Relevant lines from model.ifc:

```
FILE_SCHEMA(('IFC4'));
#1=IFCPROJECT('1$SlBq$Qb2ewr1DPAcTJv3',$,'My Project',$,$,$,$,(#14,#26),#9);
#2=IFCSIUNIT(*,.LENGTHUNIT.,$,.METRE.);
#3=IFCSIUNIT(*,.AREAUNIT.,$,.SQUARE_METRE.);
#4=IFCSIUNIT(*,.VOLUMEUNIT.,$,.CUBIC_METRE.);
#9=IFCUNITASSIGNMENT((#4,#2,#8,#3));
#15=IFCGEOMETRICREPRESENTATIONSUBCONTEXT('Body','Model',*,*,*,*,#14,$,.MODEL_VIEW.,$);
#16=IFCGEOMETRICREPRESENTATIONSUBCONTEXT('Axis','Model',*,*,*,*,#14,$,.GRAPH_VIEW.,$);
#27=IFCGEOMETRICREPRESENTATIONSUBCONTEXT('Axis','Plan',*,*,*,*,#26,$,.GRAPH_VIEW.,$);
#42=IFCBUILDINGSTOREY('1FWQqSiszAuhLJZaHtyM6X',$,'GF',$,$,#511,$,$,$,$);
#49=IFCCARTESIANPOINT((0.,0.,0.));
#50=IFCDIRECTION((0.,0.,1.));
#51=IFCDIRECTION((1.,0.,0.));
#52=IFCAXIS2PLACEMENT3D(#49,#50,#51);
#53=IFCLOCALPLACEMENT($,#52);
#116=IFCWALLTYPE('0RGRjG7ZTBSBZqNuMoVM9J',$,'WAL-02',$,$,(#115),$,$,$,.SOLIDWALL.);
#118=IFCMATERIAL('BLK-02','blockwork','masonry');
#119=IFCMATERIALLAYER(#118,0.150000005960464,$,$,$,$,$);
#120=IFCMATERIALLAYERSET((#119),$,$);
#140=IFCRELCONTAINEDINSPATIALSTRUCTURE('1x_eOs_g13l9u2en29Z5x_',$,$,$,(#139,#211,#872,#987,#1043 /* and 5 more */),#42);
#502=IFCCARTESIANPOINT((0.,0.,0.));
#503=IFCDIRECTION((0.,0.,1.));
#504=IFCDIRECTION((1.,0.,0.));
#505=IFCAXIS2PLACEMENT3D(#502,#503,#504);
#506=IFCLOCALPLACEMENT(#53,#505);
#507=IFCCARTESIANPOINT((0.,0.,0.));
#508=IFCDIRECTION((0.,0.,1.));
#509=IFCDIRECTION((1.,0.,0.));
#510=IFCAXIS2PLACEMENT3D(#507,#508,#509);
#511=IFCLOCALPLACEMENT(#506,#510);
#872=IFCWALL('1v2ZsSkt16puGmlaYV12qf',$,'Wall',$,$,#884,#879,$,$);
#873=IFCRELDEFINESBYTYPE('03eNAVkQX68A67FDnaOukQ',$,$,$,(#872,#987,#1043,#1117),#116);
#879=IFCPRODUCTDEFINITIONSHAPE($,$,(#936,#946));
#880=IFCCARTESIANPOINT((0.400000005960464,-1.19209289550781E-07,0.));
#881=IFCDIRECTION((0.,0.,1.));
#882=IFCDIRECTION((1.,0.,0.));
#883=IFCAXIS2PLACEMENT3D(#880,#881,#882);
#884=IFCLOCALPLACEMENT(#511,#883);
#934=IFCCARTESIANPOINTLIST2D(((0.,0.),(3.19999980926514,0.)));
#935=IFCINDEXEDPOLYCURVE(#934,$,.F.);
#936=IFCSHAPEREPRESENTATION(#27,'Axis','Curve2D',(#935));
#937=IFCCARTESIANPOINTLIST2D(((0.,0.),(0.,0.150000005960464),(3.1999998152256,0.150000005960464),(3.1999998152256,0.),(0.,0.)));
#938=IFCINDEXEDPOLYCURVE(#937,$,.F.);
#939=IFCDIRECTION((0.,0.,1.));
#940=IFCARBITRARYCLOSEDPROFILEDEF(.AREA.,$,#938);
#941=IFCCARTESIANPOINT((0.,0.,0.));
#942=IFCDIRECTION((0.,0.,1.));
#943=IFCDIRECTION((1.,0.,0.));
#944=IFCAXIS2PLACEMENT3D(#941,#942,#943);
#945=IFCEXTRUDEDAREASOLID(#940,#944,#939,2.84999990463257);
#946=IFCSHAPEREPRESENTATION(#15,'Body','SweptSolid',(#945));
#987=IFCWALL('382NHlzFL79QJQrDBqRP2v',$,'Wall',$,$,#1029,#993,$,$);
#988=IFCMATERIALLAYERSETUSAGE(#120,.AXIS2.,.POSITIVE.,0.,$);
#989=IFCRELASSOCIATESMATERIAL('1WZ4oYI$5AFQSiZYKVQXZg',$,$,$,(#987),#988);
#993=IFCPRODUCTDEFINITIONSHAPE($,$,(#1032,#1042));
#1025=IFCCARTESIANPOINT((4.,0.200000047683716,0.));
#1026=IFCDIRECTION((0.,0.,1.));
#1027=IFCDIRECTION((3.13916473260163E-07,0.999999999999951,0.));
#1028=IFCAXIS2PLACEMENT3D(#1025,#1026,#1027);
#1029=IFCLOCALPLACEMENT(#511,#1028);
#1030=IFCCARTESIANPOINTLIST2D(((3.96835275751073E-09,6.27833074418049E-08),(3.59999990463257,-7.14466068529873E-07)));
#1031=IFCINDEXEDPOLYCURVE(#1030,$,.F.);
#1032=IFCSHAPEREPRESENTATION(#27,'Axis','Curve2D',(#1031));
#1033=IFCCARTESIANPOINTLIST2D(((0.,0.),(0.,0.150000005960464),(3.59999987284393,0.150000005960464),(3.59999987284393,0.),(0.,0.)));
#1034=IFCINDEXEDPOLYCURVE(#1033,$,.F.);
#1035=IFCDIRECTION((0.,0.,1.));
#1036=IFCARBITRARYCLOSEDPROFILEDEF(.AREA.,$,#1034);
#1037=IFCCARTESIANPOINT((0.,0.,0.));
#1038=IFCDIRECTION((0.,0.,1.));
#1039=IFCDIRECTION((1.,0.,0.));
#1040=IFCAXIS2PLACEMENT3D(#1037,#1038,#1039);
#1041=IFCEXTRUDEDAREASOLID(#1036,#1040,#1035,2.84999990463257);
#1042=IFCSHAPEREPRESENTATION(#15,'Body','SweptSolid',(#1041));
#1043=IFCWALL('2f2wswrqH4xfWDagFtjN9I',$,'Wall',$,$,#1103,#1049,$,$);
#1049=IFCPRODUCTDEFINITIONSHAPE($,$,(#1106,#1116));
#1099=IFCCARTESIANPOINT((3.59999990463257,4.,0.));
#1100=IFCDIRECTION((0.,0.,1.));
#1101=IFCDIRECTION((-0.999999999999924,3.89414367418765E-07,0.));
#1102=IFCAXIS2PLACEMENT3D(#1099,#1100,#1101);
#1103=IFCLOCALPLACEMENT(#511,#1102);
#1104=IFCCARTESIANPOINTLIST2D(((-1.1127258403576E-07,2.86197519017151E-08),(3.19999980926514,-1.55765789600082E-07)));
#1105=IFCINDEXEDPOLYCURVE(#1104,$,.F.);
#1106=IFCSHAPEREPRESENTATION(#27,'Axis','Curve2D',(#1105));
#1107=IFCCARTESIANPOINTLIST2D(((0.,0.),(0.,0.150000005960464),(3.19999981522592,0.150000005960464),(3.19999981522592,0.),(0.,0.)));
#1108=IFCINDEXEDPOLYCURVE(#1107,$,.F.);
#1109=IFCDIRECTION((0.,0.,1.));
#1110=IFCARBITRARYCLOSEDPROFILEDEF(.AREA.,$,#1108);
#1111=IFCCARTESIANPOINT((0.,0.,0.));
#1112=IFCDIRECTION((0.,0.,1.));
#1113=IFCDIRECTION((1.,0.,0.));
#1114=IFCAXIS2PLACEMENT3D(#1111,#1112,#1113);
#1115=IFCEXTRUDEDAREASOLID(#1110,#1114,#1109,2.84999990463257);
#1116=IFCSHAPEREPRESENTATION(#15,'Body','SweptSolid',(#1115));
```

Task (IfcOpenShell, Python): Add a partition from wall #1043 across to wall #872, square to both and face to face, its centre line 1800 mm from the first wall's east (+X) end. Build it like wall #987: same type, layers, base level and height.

```python
import numpy as np
import ifcopenshell
import ifcopenshell.api.geometry
import ifcopenshell.api.material
import ifcopenshell.api.pset
import ifcopenshell.api.root
import ifcopenshell.api.spatial
import ifcopenshell.api.type
import ifcopenshell.geom
import ifcopenshell.util.element
import ifcopenshell.util.placement
import ifcopenshell.util.representation
import ifcopenshell.util.shape
import ifcopenshell.util.unit

model = ifcopenshell.open("model.ifc")
unit_scale = ifcopenshell.util.unit.calculate_unit_scale(model)
settings = ifcopenshell.geom.settings()
settings.set("use-world-coords", True)

start_wall = model.by_guid("2f2wswrqH4xfWDagFtjN9I")
end_wall = model.by_guid("1v2ZsSkt16puGmlaYV12qf")
like = model.by_guid("382NHlzFL79QJQrDBqRP2v")
matrix = ifcopenshell.util.placement.get_local_placement(start_wall.ObjectPlacement)
matrix[:3, 3] *= unit_scale


def extent(element):
    """Bounding box in the first wall's axes, in metres."""
    shape = ifcopenshell.geom.create_shape(settings, element)
    points = (ifcopenshell.util.shape.get_vertices(shape.geometry) - matrix[:3, 3]) @ matrix[:3, :3]
    return points.min(axis=0), points.max(axis=0)


y_start = extent(start_wall)[1][1]
y_end = extent(end_wall)[0][1]
like_min, like_max = extent(like)
length, height = float(abs(y_end - y_start)), float(like_max[2] - like_min[2])
layer_set = ifcopenshell.util.element.get_material(like, should_skip_usage=True)
thickness = sum(layer.LayerThickness for layer in layer_set.MaterialLayers) * unit_scale

wall = ifcopenshell.api.root.create_entity(model, ifc_class="IfcWall", name="New partition")
storey = ifcopenshell.util.element.get_container(like)
ifcopenshell.api.spatial.assign_container(model, products=[wall], relating_structure=storey)
ifcopenshell.api.type.assign_type(
    model, related_objects=[wall], relating_type=ifcopenshell.util.element.get_type(like), should_map_representations=False
)
rel = ifcopenshell.api.material.assign_material(
    model, products=[wall], type="IfcMaterialLayerSetUsage", material=layer_set
)
rel.RelatingMaterial.OffsetFromReferenceLine = -thickness / 2 / unit_scale
pset = ifcopenshell.api.pset.add_pset(model, product=wall, name="Pset_WallCommon")
ifcopenshell.api.pset.edit_pset(model, pset=pset, properties={"IsExternal": False, "LoadBearing": False})

# The axis runs down the middle of the wall.
axis = ifcopenshell.api.geometry.add_axis_representation(
    model, context=ifcopenshell.util.representation.get_context(model, "Model", "Axis"), axis=[(0.0, 0.0), (length, 0.0)]
)
body = ifcopenshell.api.geometry.add_wall_representation(
    model,
    context=ifcopenshell.util.representation.get_context(model, "Model", "Body", "MODEL_VIEW"),
    length=length,
    height=height,
    thickness=thickness,
    offset=-thickness / 2,
)
for representation in (axis, body):
    ifcopenshell.api.geometry.assign_representation(model, product=wall, representation=representation)

placement = matrix @ ifcopenshell.util.placement.rotation(90, "Z")
placement[:, 3] = matrix @ np.array([extent(start_wall)[0][0] + 1.8, y_start, like_min[2], 1.0])
ifcopenshell.api.geometry.edit_object_placement(model, product=wall, matrix=placement)

print(f"partition {length:.3f} m long, {height:.3f} m high, {thickness:.3f} m thick")

model.write("model_updated.ifc")
```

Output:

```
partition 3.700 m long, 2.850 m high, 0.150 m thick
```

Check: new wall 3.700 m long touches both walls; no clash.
